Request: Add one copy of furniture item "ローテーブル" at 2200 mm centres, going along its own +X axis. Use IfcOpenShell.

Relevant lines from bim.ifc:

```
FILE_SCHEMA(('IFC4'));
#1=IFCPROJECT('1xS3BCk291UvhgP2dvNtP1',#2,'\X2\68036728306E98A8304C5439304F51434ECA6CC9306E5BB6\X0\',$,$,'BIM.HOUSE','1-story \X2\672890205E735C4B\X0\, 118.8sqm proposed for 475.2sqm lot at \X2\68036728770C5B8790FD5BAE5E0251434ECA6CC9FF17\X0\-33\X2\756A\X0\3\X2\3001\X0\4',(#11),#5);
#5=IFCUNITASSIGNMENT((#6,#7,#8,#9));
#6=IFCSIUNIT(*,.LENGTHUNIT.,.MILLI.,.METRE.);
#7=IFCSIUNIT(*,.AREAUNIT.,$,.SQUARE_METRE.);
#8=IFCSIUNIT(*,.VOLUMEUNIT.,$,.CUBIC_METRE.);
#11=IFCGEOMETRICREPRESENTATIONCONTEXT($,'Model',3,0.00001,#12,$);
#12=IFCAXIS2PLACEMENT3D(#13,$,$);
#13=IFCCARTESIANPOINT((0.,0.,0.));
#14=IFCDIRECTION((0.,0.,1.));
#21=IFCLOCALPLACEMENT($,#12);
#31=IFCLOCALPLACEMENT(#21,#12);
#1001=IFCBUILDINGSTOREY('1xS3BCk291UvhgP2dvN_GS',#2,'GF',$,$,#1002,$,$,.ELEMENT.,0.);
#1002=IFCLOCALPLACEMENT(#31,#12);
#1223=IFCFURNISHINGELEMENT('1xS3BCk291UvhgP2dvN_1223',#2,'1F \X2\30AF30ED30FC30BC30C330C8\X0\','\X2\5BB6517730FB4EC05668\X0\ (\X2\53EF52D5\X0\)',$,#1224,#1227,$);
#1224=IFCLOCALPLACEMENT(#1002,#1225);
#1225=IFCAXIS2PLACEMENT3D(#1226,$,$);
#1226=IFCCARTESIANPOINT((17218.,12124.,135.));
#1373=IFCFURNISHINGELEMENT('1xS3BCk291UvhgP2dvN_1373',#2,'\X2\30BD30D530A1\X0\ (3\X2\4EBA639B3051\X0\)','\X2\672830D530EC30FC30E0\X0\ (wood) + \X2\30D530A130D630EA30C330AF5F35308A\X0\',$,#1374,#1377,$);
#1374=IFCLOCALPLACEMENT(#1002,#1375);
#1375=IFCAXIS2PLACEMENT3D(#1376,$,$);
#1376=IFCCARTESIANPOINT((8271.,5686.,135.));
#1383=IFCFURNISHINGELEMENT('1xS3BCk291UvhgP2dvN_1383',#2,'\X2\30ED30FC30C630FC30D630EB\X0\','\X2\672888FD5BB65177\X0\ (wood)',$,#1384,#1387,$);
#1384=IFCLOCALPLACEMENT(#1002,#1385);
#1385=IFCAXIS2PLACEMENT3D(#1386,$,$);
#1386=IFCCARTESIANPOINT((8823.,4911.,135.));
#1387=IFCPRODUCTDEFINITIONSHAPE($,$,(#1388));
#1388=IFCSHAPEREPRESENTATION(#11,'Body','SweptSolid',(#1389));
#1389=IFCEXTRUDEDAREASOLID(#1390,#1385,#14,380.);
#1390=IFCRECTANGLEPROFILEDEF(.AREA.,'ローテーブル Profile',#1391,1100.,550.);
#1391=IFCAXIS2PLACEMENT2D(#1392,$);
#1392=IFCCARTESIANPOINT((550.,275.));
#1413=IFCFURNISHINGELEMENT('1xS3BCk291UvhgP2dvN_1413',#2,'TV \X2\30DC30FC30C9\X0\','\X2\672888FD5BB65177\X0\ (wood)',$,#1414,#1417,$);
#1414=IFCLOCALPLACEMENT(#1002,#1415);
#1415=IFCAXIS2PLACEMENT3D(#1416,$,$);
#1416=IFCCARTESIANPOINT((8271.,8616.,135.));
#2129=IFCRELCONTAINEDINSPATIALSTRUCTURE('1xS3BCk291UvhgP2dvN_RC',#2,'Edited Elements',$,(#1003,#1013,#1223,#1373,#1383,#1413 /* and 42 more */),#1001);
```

```python
import ifcopenshell
import ifcopenshell.api.geometry
import ifcopenshell.api.root
import ifcopenshell.util.element
import ifcopenshell.util.placement

model = ifcopenshell.open("bim.ifc")


def reuse_history(source, copy):
    """copy_class also copies each property set's owner history, people and application; keep the originals."""
    for rel in copy.IsDefinedBy:
        if rel.is_a("IfcRelDefinesByProperties") and (history := rel.RelatingPropertyDefinition.OwnerHistory):
            rel.RelatingPropertyDefinition.OwnerHistory = source.OwnerHistory
            ifcopenshell.util.element.remove_deep2(model, history)


source = model.by_guid("1xS3BCk291UvhgP2dvN_1383")
base = ifcopenshell.util.placement.get_local_placement(source.ObjectPlacement)
step = base[:3, 0] * 2200.0

for i in range(1, 2):
    copy = ifcopenshell.api.root.copy_class(model, product=source)
    copy.Representation = ifcopenshell.util.element.copy_deep(
        model, source.Representation, exclude=["IfcGeometricRepresentationContext", "IfcRepresentationMap"]
    )
    reuse_history(source, copy)
    matrix = base.copy()
    matrix[:3, 3] += i * step
    print("added at", matrix[:3, 3].round(3) + 0.0)
    ifcopenshell.api.geometry.edit_object_placement(model, product=copy, matrix=matrix, is_si=False)

model.write("bim_updated.ifc")
```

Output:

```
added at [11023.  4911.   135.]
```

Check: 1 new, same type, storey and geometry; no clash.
